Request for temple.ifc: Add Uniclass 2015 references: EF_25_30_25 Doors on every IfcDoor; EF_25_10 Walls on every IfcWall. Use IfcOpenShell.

First a look at what the model holds.

```python
import ifcopenshell

model = ifcopenshell.open("temple.ifc")
print(model.schema)
print("classifications:", [c.Name for c in model.by_type("IfcClassification")])
for ifc_class in ("IfcDoor", "IfcRoof", "IfcStair", "IfcWall", "IfcWindow"):
    print(ifc_class, len(model.by_type(ifc_class)))
```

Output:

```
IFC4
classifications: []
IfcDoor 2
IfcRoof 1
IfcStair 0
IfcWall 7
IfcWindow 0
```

```python
import ifcopenshell
import ifcopenshell.api.classification

model = ifcopenshell.open("temple.ifc")

system = ifcopenshell.api.classification.add_classification(model, classification="Uniclass 2015")

codes = {
    "IfcDoor": ("EF_25_30_25", "Doors"),
    "IfcWall": ("EF_25_10", "Walls"),
}
for ifc_class, (code, name) in codes.items():
    products = model.by_type(ifc_class)
    ifcopenshell.api.classification.add_reference(
        model, products=products, classification=system, identification=code, name=name
    )
    print(code, len(products))

model.write("temple_updated.ifc")
```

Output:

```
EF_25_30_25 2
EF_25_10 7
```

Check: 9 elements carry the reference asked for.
